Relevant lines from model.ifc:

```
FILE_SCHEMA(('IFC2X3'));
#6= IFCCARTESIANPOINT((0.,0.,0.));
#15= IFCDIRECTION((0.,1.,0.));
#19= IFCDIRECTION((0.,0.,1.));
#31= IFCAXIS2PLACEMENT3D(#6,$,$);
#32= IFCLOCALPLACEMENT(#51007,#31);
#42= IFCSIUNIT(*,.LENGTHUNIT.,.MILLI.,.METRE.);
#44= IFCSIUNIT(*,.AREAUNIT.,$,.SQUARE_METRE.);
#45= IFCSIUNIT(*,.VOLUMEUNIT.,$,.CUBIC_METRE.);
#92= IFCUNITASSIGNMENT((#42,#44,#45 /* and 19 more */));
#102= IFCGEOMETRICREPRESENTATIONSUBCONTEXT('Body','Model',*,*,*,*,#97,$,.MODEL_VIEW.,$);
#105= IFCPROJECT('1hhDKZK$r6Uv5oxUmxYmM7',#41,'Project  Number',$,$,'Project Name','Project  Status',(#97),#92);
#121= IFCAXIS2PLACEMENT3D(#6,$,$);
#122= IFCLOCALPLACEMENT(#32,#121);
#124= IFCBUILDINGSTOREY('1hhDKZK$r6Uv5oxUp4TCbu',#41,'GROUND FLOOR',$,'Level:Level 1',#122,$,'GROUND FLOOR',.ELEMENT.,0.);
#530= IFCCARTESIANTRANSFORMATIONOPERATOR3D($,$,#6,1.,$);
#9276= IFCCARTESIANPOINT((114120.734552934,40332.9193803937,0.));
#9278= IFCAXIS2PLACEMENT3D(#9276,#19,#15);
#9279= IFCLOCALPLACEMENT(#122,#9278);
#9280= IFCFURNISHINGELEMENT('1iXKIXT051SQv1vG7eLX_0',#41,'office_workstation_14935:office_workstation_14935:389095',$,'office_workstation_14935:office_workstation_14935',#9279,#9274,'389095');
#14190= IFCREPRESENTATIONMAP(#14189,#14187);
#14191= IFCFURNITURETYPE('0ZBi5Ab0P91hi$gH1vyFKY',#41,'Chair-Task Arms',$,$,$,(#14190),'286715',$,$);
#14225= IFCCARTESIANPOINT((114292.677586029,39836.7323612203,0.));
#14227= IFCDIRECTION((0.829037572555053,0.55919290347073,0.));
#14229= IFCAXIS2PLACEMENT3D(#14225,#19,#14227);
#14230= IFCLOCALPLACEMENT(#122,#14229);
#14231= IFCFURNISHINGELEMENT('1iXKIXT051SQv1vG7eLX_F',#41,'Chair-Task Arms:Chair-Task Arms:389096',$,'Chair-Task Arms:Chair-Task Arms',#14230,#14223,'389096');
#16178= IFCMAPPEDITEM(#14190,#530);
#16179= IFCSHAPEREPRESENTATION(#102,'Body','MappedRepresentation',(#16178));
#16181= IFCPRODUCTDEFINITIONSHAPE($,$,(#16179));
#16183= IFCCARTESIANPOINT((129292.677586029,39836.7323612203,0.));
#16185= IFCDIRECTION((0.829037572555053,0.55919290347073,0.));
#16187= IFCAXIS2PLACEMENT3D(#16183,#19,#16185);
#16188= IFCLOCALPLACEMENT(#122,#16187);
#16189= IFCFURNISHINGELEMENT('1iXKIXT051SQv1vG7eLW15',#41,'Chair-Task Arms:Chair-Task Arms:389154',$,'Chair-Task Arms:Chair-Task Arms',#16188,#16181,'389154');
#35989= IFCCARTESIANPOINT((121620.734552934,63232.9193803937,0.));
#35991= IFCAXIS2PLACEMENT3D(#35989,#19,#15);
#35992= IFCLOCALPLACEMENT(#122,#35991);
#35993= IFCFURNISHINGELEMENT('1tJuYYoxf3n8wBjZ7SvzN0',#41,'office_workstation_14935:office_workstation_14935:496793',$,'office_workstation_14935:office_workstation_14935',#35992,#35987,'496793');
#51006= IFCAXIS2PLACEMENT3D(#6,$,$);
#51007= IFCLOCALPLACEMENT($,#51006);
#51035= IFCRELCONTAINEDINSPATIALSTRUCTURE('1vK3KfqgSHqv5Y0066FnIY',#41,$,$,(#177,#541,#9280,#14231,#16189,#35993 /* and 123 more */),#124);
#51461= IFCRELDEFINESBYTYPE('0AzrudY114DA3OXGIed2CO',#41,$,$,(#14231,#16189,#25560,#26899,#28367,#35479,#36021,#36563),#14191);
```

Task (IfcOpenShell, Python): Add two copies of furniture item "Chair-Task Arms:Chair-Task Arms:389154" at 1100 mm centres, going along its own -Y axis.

```python
import ifcopenshell
import ifcopenshell.api.geometry
import ifcopenshell.api.root
import ifcopenshell.util.element
import ifcopenshell.util.placement

model = ifcopenshell.open("model.ifc")


def reuse_history(source, copy):
    """copy_class also copies each property set's owner history, people and application; keep the originals."""
    for rel in copy.IsDefinedBy:
        if rel.is_a("IfcRelDefinesByProperties") and (history := rel.RelatingPropertyDefinition.OwnerHistory):
            rel.RelatingPropertyDefinition.OwnerHistory = source.OwnerHistory
            ifcopenshell.util.element.remove_deep2(model, history)


source = model.by_guid("1iXKIXT051SQv1vG7eLW15")
base = ifcopenshell.util.placement.get_local_placement(source.ObjectPlacement)
step = -base[:3, 1] * 1100.0

for i in range(1, 3):
    copy = ifcopenshell.api.root.copy_class(model, product=source)
    copy.Representation = ifcopenshell.util.element.copy_deep(
        model, source.Representation, exclude=["IfcGeometricRepresentationContext", "IfcRepresentationMap"]
    )
    copy.Name = "Chair-Task Arms:Chair-Task Arms"
    copy.Tag = None
    reuse_history(source, copy)
    matrix = base.copy()
    matrix[:3, 3] += i * step
    print("added at", matrix[:3, 3].round(3) + 0.0)
    ifcopenshell.api.geometry.edit_object_placement(model, product=copy, matrix=matrix, is_si=False)

model.write("model_rev.ifc")
```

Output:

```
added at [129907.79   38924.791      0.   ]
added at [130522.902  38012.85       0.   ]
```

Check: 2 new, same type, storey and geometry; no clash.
